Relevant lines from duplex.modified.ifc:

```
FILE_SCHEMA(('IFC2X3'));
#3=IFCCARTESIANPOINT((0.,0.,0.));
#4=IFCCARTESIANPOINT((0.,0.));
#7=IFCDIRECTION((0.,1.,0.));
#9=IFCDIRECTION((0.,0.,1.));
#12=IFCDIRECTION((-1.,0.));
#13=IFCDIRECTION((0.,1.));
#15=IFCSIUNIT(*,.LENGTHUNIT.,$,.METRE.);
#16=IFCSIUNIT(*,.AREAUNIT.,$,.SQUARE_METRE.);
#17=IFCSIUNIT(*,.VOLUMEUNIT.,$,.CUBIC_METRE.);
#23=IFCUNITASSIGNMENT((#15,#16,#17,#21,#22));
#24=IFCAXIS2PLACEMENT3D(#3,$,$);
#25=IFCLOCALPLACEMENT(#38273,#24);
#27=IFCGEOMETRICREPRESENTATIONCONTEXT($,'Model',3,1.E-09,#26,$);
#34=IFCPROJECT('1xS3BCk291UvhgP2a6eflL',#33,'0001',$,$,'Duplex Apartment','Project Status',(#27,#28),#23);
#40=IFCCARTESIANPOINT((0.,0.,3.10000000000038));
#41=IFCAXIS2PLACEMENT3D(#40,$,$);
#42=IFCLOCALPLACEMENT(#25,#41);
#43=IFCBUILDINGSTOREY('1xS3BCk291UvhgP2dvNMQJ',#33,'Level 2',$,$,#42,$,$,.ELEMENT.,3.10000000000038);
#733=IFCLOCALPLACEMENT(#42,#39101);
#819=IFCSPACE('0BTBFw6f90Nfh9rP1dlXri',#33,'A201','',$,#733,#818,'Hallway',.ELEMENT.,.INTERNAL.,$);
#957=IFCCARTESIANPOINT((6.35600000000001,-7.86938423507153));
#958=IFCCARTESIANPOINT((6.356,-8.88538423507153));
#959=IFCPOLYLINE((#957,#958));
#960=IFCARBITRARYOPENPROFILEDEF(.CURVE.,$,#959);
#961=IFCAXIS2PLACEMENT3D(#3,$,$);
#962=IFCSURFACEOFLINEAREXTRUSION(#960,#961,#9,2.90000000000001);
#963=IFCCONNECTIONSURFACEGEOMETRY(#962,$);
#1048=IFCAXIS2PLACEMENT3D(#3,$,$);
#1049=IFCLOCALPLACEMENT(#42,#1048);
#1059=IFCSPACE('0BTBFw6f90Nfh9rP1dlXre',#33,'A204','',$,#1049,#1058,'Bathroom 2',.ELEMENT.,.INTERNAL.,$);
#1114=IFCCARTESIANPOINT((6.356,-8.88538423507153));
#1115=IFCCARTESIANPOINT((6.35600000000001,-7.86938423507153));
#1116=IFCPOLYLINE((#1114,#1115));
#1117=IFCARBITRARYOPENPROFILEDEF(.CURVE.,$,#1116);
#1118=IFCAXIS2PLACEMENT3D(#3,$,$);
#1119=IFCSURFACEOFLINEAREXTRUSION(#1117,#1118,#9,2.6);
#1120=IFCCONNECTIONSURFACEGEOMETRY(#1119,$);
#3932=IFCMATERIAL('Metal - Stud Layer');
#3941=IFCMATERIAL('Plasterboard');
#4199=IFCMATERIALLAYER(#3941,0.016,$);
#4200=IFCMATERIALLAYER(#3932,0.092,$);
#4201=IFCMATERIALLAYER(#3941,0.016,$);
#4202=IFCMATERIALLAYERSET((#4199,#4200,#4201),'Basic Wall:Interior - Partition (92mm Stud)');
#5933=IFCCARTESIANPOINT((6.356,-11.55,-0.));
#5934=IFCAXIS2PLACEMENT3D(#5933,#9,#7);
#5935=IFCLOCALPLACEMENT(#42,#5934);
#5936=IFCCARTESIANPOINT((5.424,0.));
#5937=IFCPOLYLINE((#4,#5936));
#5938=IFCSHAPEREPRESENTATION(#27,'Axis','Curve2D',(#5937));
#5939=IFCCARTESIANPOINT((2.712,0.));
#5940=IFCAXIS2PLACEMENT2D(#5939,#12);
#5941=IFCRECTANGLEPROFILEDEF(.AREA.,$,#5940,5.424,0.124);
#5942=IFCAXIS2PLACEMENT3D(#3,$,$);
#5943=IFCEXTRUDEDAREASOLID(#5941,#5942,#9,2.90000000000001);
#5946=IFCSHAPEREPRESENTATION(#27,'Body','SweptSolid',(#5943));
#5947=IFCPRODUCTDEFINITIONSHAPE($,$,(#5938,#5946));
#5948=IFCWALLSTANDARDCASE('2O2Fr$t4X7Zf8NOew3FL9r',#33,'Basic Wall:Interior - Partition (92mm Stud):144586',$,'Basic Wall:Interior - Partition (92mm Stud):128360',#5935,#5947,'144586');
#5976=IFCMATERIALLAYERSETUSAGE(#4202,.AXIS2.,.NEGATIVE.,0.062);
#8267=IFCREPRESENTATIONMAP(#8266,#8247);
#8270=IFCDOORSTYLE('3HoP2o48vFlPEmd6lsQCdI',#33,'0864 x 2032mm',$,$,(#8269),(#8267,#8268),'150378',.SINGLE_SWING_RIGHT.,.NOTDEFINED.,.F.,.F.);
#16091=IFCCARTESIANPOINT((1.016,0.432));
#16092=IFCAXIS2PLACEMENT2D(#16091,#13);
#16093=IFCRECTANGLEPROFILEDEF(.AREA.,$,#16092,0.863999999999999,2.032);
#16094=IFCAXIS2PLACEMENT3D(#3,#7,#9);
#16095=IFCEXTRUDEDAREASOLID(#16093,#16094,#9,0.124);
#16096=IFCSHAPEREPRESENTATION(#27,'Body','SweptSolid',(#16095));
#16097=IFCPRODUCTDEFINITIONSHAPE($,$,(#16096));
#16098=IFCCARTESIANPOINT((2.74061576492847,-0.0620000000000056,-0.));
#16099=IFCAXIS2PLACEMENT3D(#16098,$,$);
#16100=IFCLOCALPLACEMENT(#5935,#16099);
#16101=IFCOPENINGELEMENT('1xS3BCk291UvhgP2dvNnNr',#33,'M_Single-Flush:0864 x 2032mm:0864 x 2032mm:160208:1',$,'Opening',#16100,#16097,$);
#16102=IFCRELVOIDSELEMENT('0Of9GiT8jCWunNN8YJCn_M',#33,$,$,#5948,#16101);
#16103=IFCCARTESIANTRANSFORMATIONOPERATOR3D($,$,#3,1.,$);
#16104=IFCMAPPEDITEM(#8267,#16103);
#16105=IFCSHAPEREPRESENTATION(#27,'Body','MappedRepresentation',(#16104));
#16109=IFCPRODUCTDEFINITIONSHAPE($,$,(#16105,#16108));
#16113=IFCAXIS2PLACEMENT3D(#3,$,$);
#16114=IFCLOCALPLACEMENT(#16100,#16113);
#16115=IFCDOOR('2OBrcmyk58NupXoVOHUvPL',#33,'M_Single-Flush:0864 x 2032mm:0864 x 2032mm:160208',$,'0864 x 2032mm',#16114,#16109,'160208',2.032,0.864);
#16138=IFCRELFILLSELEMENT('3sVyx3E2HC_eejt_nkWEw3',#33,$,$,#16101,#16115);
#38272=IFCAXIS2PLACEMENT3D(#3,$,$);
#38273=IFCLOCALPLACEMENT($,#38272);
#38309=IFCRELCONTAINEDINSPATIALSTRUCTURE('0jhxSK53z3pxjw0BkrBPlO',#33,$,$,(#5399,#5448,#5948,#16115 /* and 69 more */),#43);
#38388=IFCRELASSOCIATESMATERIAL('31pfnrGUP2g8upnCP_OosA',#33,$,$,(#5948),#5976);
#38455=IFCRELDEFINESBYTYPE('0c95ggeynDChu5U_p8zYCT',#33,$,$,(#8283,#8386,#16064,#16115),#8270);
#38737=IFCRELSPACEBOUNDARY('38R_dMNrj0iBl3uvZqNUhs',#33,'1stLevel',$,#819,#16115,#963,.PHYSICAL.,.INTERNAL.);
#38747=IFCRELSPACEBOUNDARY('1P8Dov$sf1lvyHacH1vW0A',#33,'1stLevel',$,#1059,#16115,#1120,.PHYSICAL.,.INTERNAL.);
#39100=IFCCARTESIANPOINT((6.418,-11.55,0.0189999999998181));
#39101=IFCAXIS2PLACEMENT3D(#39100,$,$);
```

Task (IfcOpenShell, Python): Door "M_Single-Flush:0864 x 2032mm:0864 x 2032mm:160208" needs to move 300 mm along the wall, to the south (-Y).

```python
import numpy as np
import ifcopenshell
import ifcopenshell.api.geometry
import ifcopenshell.util.placement
import ifcopenshell.util.unit

model = ifcopenshell.open("duplex.modified.ifc")
unit_scale = ifcopenshell.util.unit.calculate_unit_scale(model)

door = model.by_guid("2OBrcmyk58NupXoVOHUvPL")
opening = door.FillsVoids[0].RelatingOpeningElement
wall = opening.VoidsElements[0].RelatingBuildingElement

wall_matrix = ifcopenshell.util.placement.get_local_placement(wall.ObjectPlacement)
shift = wall_matrix[:3, 0] * -0.3 / unit_scale
before = ifcopenshell.util.placement.get_local_placement(door.ObjectPlacement)[:3, 3].copy()

# The door is placed relative to its opening, so it follows when the opening moves.
matrix = ifcopenshell.util.placement.get_local_placement(opening.ObjectPlacement)
matrix[:3, 3] += shift
ifcopenshell.api.geometry.edit_object_placement(
    model, product=opening, matrix=matrix, is_si=False, should_transform_children=True
)

# Space boundary surfaces are stored in each space's coordinates; move them too.
for rel in door.ProvidesBoundaries:
    if not rel.ConnectionGeometry:
        continue
    surface = rel.ConnectionGeometry.SurfaceOnRelatingElement
    space_matrix = ifcopenshell.util.placement.get_local_placement(rel.RelatingSpace.ObjectPlacement)
    point = np.array(surface.Position.Location.Coordinates) + space_matrix[:3, :3].T @ shift
    surface.Position = model.createIfcAxis2Placement3D(
        model.createIfcCartesianPoint(point.tolist()), surface.Position.Axis, surface.Position.RefDirection
    )

after = ifcopenshell.util.placement.get_local_placement(door.ObjectPlacement)[:3, 3]
print("door moved by", (after - before).round(3) + 0.0)

model.write("duplex.modified-out.ifc")
```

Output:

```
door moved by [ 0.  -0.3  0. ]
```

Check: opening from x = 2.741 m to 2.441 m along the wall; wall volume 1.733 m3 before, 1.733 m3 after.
